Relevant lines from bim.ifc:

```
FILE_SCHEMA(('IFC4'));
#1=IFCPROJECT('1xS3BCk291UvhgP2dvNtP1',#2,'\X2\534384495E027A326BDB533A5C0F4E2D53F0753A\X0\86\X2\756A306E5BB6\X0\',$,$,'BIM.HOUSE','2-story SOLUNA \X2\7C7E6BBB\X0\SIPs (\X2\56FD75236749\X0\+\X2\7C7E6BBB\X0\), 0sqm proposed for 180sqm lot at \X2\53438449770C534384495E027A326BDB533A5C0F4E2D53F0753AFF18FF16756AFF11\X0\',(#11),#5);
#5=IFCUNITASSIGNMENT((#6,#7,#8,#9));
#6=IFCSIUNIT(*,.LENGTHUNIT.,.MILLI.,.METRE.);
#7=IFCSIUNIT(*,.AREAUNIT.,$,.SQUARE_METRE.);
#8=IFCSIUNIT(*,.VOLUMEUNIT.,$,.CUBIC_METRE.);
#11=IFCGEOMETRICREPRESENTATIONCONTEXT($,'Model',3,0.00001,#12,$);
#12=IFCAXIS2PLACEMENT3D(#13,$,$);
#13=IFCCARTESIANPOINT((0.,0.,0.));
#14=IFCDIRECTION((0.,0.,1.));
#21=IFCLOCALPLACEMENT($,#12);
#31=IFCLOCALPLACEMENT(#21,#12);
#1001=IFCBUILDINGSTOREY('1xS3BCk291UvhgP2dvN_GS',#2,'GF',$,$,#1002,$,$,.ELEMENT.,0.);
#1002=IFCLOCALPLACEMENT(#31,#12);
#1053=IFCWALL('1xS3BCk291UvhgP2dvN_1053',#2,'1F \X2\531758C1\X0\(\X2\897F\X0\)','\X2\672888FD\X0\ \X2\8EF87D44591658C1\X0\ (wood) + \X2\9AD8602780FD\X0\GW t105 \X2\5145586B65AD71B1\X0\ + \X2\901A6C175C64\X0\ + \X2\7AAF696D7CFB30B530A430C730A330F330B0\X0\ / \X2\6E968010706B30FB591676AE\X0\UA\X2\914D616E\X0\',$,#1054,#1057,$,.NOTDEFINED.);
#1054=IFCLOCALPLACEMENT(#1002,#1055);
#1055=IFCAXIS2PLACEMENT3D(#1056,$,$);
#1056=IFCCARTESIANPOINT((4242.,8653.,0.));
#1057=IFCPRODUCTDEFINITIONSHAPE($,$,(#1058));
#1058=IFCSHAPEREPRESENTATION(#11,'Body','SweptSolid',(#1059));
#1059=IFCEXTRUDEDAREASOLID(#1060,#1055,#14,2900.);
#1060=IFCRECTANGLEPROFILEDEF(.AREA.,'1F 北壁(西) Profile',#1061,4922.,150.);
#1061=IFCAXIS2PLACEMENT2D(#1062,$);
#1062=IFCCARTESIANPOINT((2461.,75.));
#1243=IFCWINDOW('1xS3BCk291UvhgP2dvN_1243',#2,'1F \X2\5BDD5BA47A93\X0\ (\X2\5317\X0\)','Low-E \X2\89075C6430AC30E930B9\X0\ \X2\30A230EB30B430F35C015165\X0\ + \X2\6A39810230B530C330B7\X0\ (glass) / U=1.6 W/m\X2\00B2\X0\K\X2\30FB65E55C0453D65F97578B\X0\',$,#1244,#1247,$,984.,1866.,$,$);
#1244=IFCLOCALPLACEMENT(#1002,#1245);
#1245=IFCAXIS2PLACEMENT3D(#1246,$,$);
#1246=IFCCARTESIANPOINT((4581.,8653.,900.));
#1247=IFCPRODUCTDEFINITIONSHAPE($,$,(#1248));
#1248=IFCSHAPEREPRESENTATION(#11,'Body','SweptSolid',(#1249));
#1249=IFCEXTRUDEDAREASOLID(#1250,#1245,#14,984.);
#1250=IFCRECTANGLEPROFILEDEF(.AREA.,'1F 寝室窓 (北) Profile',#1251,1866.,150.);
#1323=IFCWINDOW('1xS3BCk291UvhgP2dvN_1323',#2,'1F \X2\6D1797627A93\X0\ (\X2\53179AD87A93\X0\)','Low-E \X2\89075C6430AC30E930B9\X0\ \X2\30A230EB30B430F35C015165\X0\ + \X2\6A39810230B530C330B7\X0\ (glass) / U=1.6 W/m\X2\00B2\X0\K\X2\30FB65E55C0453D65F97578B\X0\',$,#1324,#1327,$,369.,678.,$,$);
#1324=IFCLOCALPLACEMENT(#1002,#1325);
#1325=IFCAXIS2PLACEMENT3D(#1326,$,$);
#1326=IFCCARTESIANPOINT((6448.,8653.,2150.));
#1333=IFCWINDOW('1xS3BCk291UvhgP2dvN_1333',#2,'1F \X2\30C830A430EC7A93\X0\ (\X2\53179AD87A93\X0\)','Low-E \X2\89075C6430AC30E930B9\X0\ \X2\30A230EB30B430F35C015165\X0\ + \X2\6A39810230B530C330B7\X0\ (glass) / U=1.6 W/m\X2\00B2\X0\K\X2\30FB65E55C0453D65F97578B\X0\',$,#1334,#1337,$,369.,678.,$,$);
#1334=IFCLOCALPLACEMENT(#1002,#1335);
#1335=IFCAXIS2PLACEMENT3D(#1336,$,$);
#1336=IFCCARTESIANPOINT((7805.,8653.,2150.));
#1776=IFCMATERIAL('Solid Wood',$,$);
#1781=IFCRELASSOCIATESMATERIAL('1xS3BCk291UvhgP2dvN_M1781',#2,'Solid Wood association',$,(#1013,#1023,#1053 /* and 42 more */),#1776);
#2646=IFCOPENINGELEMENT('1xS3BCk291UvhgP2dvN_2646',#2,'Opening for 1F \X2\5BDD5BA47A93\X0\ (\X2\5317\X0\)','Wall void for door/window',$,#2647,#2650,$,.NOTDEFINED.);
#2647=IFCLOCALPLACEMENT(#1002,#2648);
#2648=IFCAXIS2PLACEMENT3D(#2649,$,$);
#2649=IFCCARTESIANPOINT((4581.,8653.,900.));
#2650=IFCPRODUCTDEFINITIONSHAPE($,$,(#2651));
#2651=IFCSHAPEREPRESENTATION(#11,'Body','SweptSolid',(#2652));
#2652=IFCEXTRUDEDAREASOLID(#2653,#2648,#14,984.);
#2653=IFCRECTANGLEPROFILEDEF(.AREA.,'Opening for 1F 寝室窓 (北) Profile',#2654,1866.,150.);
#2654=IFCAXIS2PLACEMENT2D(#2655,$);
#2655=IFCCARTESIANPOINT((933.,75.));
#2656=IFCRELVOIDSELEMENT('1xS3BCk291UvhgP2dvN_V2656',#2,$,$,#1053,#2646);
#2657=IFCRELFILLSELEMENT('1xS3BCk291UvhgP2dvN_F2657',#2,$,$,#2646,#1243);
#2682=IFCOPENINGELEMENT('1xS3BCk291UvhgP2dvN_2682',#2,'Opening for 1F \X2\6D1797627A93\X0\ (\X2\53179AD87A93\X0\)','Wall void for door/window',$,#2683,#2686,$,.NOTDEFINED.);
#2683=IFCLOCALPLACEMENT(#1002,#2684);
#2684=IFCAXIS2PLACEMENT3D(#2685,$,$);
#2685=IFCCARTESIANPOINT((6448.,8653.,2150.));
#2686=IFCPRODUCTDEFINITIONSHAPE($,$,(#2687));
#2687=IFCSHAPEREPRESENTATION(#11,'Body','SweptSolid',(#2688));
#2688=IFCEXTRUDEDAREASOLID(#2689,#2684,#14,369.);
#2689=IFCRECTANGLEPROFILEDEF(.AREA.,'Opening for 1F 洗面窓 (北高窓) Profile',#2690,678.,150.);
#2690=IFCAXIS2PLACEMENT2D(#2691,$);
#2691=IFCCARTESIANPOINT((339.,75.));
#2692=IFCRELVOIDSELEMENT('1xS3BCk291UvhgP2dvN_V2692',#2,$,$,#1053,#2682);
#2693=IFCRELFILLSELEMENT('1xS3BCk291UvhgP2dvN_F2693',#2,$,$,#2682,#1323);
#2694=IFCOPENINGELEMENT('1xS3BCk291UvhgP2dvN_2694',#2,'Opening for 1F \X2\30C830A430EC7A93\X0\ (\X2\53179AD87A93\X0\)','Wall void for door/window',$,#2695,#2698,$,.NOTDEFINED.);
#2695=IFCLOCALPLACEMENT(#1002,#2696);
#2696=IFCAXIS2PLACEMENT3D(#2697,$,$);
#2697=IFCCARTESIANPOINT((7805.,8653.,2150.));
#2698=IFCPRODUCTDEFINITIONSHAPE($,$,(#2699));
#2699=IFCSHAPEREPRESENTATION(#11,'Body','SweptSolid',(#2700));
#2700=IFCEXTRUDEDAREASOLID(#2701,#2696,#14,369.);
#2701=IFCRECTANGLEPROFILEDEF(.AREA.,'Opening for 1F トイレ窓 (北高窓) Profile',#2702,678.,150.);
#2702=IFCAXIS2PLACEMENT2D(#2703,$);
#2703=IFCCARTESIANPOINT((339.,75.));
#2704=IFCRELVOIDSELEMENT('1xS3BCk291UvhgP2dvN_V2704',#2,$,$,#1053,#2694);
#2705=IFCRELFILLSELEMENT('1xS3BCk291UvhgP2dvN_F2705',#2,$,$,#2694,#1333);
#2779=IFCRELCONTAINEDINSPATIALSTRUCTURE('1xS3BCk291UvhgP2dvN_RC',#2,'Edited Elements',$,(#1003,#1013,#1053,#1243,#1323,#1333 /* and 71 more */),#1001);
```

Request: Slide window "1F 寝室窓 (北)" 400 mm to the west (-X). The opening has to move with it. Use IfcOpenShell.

```python
import ifcopenshell
import ifcopenshell.api.geometry
import ifcopenshell.util.placement
import ifcopenshell.util.unit

model = ifcopenshell.open("bim.ifc")
unit_scale = ifcopenshell.util.unit.calculate_unit_scale(model)

window = model.by_guid("1xS3BCk291UvhgP2dvN_1243")
opening = window.FillsVoids[0].RelatingOpeningElement
wall = opening.VoidsElements[0].RelatingBuildingElement

wall_matrix = ifcopenshell.util.placement.get_local_placement(wall.ObjectPlacement)
shift = wall_matrix[:3, 0] * -0.4 / unit_scale
before = ifcopenshell.util.placement.get_local_placement(window.ObjectPlacement)[:3, 3].copy()

# The window is not placed relative to its opening, so move both.
for product in (opening, window):
    matrix = ifcopenshell.util.placement.get_local_placement(product.ObjectPlacement)
    matrix[:3, 3] += shift
    ifcopenshell.api.geometry.edit_object_placement(model, product=product, matrix=matrix, is_si=False)

after = ifcopenshell.util.placement.get_local_placement(window.ObjectPlacement)[:3, 3]
print("window moved by", (after - before).round(3) + 0.0)

model.write("bim_updated.ifc")
```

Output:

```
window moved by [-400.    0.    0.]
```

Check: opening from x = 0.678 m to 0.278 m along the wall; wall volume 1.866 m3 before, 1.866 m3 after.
